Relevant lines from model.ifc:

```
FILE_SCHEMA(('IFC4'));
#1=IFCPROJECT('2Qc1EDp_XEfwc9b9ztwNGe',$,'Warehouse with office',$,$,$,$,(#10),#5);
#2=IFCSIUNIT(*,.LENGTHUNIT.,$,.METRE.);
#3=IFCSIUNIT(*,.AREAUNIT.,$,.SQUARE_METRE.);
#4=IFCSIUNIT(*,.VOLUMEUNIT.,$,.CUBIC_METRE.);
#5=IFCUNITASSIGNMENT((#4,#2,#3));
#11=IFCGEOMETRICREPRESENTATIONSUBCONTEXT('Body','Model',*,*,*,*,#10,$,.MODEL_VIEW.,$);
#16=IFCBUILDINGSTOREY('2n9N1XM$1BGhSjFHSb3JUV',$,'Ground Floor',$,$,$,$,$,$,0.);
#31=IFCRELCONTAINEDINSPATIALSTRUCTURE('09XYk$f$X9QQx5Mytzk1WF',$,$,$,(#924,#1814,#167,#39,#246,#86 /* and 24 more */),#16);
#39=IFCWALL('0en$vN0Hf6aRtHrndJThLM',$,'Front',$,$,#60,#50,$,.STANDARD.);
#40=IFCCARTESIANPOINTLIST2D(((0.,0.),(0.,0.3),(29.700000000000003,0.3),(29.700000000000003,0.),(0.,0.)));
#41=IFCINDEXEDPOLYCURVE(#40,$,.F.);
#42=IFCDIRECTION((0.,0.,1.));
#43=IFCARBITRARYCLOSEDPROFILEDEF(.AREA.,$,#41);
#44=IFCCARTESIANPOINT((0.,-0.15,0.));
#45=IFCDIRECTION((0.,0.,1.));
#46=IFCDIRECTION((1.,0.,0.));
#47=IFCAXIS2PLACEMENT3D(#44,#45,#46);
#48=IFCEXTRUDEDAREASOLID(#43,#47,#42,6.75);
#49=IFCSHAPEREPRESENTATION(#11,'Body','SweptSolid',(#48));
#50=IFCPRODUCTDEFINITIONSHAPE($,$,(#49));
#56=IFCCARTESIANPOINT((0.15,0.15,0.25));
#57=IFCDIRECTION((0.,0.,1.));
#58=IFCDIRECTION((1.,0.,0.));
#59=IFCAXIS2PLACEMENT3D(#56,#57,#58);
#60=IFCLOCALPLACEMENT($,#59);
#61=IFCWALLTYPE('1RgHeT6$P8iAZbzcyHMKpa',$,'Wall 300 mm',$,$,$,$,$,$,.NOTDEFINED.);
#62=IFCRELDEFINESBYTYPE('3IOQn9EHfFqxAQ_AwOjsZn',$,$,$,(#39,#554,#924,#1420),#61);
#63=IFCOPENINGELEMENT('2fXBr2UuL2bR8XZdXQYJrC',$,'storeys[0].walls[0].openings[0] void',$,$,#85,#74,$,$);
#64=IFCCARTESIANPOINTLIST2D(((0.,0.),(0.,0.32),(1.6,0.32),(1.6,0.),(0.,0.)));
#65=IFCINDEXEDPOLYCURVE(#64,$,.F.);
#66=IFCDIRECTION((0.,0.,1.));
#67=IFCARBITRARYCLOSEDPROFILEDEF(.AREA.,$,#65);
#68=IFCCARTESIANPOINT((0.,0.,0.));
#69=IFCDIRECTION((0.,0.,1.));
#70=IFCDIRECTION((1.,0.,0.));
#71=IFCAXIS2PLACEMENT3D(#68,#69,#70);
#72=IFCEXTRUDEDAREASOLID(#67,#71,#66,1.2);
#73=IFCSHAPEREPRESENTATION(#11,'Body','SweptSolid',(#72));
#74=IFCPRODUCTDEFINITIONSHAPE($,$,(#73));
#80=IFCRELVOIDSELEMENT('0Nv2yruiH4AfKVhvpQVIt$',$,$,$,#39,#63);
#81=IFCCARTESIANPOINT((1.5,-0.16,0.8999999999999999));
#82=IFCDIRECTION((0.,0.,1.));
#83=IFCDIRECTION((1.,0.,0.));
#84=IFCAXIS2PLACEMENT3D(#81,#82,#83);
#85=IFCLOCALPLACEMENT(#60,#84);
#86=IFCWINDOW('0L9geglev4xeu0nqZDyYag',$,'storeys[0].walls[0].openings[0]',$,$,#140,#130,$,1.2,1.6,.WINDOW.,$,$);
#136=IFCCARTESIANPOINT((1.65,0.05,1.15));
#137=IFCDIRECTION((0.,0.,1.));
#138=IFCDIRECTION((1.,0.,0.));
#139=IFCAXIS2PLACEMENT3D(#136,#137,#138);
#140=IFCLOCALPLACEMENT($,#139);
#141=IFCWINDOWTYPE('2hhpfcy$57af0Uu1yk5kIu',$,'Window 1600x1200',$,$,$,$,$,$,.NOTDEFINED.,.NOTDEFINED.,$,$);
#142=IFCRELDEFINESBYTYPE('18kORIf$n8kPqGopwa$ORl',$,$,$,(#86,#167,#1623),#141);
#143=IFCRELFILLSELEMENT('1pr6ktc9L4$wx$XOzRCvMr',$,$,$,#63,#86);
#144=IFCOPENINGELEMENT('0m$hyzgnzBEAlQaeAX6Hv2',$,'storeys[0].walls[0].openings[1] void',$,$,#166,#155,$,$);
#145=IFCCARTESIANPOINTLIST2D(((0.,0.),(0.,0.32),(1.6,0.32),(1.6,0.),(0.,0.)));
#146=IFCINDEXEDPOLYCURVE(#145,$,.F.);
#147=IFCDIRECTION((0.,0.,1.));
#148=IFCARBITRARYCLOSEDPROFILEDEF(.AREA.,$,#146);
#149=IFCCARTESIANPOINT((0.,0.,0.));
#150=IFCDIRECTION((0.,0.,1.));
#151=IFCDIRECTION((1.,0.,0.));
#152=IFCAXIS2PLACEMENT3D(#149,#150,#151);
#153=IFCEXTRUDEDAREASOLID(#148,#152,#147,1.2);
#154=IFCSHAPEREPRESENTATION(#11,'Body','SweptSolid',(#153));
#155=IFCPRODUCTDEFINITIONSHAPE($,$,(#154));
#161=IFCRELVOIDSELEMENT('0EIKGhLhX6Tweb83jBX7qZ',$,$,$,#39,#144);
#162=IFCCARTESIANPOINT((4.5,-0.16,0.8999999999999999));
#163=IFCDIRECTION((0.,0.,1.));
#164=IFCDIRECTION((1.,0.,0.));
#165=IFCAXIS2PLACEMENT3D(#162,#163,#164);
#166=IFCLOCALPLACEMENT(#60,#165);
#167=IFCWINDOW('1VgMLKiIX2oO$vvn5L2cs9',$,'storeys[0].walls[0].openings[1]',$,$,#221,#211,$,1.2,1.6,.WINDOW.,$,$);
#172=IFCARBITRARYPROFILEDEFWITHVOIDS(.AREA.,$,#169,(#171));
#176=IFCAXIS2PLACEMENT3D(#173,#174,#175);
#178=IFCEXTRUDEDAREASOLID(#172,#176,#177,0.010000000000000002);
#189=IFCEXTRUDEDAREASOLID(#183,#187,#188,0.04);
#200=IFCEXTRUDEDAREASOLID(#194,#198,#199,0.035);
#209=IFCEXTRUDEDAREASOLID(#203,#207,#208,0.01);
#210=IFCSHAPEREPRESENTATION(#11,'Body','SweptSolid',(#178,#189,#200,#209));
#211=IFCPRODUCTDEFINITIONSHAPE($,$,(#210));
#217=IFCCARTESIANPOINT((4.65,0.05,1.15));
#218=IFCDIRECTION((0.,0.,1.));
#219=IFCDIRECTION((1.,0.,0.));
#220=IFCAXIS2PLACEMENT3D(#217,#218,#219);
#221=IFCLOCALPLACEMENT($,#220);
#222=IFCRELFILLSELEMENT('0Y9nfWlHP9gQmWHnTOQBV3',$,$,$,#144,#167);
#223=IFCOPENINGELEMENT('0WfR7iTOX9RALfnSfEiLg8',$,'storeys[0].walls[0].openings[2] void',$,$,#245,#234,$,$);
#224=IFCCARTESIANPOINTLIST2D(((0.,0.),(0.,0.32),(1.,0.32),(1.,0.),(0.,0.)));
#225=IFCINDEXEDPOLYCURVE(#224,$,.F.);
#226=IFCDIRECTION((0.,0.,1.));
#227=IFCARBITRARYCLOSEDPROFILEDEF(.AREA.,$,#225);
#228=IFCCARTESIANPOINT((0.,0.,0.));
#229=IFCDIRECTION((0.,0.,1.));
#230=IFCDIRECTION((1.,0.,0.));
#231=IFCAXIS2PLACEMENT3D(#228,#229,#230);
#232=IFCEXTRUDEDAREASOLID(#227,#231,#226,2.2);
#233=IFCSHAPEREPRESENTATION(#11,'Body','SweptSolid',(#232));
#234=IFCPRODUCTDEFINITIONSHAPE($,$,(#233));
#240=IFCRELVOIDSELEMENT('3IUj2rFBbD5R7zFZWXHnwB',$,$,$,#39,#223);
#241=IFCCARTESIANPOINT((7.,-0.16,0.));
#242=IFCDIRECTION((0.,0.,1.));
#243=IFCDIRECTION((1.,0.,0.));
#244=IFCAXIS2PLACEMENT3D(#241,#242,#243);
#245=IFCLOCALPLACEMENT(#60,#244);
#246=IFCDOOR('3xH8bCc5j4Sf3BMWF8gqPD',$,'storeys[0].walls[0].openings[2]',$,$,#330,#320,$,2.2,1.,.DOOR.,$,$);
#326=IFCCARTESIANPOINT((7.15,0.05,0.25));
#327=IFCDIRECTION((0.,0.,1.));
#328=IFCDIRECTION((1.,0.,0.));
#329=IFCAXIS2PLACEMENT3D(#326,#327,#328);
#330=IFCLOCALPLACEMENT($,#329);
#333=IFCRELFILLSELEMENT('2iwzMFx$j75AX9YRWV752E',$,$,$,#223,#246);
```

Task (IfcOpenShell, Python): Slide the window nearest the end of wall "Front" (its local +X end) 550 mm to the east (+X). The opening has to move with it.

```python
import ifcopenshell
import ifcopenshell.api.geometry
import ifcopenshell.util.placement
import ifcopenshell.util.unit

model = ifcopenshell.open("model.ifc")
unit_scale = ifcopenshell.util.unit.calculate_unit_scale(model)

window = model.by_id(167)
opening = window.FillsVoids[0].RelatingOpeningElement
wall = opening.VoidsElements[0].RelatingBuildingElement

wall_matrix = ifcopenshell.util.placement.get_local_placement(wall.ObjectPlacement)
shift = wall_matrix[:3, 0] * 0.55 / unit_scale
before = ifcopenshell.util.placement.get_local_placement(window.ObjectPlacement)[:3, 3].copy()

# The window is not placed relative to its opening, so move both.
for product in (opening, window):
    matrix = ifcopenshell.util.placement.get_local_placement(product.ObjectPlacement)
    matrix[:3, 3] += shift
    ifcopenshell.api.geometry.edit_object_placement(model, product=product, matrix=matrix, is_si=False)

after = ifcopenshell.util.placement.get_local_placement(window.ObjectPlacement)[:3, 3]
print("window moved by", (after - before).round(3) + 0.0)

model.write("model_v2.ifc")
```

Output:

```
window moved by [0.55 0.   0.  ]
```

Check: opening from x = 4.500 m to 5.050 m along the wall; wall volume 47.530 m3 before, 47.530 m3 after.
